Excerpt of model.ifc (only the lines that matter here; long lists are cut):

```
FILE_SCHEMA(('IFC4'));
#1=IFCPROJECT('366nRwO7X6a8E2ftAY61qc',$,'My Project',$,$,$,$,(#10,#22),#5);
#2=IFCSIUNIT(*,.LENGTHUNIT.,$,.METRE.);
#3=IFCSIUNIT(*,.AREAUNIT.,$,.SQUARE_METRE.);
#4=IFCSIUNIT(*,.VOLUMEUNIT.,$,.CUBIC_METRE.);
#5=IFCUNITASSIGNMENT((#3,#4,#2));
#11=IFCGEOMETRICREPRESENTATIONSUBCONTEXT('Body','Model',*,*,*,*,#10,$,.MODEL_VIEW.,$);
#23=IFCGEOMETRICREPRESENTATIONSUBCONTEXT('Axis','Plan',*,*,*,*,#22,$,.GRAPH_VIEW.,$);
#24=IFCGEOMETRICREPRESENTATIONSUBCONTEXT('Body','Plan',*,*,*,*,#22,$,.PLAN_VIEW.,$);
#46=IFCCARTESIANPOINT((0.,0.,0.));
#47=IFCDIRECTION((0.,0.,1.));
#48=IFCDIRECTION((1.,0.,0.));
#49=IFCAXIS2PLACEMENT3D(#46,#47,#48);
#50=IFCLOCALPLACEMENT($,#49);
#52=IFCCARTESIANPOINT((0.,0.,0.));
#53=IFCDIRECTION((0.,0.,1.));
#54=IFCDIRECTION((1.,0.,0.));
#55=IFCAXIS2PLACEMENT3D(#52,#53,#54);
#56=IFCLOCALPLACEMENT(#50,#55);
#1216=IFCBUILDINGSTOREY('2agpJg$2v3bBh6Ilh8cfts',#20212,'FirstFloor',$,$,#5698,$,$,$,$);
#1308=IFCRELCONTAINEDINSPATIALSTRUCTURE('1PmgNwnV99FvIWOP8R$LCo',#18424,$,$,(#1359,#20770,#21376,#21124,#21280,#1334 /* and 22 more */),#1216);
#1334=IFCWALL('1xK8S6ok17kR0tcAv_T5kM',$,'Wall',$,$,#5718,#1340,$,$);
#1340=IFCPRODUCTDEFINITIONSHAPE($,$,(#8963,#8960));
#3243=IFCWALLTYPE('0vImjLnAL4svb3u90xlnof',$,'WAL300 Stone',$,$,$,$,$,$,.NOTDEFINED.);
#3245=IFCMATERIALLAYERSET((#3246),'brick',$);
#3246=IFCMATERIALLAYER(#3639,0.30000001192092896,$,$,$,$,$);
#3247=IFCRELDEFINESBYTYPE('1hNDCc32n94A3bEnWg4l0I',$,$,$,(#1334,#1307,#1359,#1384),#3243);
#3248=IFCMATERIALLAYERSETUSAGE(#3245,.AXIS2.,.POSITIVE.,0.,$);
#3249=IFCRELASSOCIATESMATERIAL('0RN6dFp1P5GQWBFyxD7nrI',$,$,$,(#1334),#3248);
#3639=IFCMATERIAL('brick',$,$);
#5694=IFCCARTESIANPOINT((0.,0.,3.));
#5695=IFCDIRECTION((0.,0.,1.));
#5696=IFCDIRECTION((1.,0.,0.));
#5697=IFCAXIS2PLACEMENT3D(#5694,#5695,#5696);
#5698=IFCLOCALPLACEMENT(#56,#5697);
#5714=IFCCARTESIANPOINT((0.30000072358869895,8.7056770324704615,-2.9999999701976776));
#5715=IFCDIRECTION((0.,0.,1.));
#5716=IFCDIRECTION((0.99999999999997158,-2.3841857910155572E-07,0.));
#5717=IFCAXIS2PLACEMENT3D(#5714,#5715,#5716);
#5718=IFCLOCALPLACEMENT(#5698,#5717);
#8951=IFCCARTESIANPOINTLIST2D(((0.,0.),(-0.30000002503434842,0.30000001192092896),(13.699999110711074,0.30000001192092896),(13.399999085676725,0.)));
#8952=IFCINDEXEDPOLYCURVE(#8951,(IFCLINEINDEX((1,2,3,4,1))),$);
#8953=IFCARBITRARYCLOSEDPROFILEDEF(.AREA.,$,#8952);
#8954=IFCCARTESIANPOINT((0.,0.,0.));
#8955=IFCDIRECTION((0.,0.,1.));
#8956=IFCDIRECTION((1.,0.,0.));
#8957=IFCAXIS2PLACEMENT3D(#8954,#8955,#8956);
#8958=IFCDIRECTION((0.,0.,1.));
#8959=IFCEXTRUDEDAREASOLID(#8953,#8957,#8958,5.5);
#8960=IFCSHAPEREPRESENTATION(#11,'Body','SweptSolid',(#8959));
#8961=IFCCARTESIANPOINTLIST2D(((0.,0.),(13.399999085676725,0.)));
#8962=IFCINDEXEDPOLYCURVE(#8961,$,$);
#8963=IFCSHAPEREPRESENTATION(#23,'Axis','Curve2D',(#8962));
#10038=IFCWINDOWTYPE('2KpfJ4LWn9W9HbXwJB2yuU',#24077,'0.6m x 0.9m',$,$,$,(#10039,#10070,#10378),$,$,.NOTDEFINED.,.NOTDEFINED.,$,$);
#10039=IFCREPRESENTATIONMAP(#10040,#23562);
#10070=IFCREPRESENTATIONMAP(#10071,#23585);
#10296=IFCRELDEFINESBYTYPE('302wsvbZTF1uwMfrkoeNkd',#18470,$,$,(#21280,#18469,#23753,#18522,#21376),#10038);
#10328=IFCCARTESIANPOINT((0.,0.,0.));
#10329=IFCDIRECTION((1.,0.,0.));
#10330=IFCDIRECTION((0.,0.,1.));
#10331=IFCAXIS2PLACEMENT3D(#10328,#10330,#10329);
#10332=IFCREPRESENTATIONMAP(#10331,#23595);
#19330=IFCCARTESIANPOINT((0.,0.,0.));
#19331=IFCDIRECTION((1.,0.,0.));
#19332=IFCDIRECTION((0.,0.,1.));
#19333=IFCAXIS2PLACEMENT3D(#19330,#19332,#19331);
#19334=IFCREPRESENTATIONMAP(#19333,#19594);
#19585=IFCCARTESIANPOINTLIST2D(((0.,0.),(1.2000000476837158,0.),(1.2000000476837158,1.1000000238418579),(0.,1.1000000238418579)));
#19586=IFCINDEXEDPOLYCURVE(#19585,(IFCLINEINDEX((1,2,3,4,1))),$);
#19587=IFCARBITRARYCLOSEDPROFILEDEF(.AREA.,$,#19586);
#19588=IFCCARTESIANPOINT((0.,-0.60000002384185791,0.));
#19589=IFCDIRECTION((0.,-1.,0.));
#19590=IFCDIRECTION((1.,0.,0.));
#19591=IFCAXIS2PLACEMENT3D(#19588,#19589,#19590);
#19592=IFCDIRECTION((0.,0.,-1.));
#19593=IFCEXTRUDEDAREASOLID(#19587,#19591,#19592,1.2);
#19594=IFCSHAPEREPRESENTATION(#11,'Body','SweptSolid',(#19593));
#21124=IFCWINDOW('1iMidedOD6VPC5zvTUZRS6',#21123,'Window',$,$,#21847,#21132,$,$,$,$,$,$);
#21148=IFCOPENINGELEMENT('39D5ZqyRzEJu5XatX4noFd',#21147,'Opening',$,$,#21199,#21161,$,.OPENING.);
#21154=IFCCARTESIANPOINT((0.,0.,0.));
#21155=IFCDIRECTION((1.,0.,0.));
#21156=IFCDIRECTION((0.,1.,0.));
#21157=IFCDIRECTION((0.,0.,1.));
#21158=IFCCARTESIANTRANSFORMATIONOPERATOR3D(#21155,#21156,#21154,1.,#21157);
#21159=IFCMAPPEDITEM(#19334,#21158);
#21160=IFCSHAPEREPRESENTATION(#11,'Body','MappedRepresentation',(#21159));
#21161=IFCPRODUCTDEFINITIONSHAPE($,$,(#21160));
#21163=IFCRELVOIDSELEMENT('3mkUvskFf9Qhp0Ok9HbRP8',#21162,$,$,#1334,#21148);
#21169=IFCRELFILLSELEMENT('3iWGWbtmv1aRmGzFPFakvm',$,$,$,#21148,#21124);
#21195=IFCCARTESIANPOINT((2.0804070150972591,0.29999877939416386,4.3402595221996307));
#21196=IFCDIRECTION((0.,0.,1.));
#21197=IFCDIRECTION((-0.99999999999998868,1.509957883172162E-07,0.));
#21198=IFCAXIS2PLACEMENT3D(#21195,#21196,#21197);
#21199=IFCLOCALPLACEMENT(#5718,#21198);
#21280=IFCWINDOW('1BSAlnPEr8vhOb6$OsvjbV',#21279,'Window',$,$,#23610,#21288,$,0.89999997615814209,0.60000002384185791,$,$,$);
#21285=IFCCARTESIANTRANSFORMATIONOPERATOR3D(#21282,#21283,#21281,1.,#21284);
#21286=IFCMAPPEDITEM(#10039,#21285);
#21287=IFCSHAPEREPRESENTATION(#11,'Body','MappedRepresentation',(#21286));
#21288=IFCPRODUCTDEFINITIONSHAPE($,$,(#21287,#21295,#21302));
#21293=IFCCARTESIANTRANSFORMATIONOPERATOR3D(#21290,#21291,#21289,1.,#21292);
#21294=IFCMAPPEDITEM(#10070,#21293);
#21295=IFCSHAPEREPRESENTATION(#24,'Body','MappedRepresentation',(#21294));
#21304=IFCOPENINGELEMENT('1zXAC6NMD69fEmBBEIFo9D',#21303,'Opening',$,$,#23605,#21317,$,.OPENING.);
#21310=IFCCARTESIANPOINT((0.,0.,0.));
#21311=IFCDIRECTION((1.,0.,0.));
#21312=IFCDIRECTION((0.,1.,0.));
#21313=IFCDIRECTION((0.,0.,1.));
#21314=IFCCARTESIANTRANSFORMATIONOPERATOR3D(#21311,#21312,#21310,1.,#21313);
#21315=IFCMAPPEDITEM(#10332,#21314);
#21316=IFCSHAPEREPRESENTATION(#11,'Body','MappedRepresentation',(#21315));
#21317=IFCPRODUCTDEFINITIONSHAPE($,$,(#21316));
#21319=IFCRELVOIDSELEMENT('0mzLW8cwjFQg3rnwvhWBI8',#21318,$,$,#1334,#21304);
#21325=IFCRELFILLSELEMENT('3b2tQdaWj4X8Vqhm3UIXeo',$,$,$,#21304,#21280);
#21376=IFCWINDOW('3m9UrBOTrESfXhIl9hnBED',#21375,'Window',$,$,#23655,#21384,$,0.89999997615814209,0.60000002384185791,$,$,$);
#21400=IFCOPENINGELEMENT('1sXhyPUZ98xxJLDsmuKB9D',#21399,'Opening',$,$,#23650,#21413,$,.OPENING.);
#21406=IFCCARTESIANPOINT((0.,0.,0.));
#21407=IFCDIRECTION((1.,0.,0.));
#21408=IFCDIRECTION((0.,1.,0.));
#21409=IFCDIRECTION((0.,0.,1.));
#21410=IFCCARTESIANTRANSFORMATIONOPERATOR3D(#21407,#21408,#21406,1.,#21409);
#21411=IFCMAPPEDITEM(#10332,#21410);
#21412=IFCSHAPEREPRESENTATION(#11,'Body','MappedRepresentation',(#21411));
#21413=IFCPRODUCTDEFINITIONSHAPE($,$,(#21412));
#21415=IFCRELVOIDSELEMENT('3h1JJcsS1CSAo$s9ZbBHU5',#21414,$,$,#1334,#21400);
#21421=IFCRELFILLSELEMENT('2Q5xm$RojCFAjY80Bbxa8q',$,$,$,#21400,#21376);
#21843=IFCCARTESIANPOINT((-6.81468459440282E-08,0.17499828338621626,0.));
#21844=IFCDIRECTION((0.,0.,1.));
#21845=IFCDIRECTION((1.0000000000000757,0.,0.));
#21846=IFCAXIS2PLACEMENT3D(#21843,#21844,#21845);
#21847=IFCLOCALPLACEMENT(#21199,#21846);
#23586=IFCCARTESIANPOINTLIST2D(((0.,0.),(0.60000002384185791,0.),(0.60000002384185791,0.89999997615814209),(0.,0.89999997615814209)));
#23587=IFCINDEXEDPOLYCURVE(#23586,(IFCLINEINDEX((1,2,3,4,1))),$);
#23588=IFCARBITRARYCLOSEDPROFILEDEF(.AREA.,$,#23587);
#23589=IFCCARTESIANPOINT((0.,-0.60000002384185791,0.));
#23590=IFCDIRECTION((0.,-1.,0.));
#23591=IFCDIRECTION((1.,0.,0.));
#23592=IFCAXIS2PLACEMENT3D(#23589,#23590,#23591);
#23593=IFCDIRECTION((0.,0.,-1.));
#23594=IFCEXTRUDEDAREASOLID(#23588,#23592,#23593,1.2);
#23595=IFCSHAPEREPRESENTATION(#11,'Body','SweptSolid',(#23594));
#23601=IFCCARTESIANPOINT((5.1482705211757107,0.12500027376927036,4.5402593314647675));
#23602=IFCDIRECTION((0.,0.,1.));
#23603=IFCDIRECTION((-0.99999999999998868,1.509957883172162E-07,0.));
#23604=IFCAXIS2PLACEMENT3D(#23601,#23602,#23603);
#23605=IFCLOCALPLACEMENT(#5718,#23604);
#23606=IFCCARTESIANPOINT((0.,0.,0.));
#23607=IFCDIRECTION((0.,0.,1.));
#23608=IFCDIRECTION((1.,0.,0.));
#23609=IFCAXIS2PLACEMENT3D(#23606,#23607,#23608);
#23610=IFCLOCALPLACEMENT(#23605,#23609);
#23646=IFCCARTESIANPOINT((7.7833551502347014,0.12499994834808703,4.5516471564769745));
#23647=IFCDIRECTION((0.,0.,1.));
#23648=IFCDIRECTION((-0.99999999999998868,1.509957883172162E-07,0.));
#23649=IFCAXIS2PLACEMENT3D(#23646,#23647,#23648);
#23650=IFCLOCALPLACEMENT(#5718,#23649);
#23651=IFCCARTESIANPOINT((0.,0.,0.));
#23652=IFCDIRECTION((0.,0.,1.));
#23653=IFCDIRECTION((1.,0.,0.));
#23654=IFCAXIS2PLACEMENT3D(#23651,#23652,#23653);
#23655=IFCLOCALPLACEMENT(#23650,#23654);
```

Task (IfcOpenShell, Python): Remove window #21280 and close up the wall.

```python
import ifcopenshell
import ifcopenshell.api.feature
import ifcopenshell.api.root
import ifcopenshell.geom
import ifcopenshell.util.shape

model = ifcopenshell.open("model.ifc")
settings = ifcopenshell.geom.settings()


def volume(element):
    """Net volume in cubic metres, openings subtracted."""
    shape = ifcopenshell.geom.create_shape(settings, element)
    return ifcopenshell.util.shape.get_volume(shape.geometry)


window = model.by_guid("1BSAlnPEr8vhOb6$OsvjbV")
opening = window.FillsVoids[0].RelatingOpeningElement
wall = opening.VoidsElements[0].RelatingBuildingElement
before = volume(wall)

ifcopenshell.api.root.remove_product(model, product=window)
ifcopenshell.api.feature.remove_feature(model, feature=opening)

after = volume(wall)

print(f"wall volume {before:.3f} -> {after:.3f} m3")

model.write("model-out.ifc")
```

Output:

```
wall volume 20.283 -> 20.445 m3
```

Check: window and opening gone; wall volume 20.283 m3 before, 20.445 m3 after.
